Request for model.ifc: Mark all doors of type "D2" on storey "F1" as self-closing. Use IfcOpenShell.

First a look at what the model holds.

```python
import ifcopenshell
import ifcopenshell.util.element

model = ifcopenshell.open("model.ifc")
print(model.schema)
storey = next(s for s in model.by_type("IfcBuildingStorey") if s.Name == "F1")
doors = [e for e in ifcopenshell.util.element.get_decomposition(storey) if e.is_a("IfcDoor")]
seen = {}
for e in doors:
    element_type = ifcopenshell.util.element.get_type(e)
    key = (element_type.Name if element_type != e and element_type else None, ifcopenshell.util.element.get_pset(e, "Pset_DoorCommon", "SelfClosing"))
    seen[key] = seen.get(key, 0) + 1
for (name, value), count in sorted(seen.items(), key=str):
    print(count, "x", name, "|", value)
```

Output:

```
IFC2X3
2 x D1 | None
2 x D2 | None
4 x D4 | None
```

```python
import ifcopenshell
import ifcopenshell.api.pset
import ifcopenshell.util.element

model = ifcopenshell.open("model.ifc")

storey = next(s for s in model.by_type("IfcBuildingStorey") if s.Name == "F1")
doors = [e for e in ifcopenshell.util.element.get_decomposition(storey) if e.is_a("IfcDoor")]

count = 0
for e in doors:
    element_type = ifcopenshell.util.element.get_type(e)
    if element_type in (None, e) or element_type.Name != "D2":
        continue
    # add_pset returns the element's existing set when there is one.
    pset = ifcopenshell.api.pset.add_pset(model, product=e, name="Pset_DoorCommon")
    ifcopenshell.api.pset.edit_pset(model, pset=pset, properties={"SelfClosing": True})
    count += 1

print(count, "doors updated")

model.write("model_rev.ifc")
```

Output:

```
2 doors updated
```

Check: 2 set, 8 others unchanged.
